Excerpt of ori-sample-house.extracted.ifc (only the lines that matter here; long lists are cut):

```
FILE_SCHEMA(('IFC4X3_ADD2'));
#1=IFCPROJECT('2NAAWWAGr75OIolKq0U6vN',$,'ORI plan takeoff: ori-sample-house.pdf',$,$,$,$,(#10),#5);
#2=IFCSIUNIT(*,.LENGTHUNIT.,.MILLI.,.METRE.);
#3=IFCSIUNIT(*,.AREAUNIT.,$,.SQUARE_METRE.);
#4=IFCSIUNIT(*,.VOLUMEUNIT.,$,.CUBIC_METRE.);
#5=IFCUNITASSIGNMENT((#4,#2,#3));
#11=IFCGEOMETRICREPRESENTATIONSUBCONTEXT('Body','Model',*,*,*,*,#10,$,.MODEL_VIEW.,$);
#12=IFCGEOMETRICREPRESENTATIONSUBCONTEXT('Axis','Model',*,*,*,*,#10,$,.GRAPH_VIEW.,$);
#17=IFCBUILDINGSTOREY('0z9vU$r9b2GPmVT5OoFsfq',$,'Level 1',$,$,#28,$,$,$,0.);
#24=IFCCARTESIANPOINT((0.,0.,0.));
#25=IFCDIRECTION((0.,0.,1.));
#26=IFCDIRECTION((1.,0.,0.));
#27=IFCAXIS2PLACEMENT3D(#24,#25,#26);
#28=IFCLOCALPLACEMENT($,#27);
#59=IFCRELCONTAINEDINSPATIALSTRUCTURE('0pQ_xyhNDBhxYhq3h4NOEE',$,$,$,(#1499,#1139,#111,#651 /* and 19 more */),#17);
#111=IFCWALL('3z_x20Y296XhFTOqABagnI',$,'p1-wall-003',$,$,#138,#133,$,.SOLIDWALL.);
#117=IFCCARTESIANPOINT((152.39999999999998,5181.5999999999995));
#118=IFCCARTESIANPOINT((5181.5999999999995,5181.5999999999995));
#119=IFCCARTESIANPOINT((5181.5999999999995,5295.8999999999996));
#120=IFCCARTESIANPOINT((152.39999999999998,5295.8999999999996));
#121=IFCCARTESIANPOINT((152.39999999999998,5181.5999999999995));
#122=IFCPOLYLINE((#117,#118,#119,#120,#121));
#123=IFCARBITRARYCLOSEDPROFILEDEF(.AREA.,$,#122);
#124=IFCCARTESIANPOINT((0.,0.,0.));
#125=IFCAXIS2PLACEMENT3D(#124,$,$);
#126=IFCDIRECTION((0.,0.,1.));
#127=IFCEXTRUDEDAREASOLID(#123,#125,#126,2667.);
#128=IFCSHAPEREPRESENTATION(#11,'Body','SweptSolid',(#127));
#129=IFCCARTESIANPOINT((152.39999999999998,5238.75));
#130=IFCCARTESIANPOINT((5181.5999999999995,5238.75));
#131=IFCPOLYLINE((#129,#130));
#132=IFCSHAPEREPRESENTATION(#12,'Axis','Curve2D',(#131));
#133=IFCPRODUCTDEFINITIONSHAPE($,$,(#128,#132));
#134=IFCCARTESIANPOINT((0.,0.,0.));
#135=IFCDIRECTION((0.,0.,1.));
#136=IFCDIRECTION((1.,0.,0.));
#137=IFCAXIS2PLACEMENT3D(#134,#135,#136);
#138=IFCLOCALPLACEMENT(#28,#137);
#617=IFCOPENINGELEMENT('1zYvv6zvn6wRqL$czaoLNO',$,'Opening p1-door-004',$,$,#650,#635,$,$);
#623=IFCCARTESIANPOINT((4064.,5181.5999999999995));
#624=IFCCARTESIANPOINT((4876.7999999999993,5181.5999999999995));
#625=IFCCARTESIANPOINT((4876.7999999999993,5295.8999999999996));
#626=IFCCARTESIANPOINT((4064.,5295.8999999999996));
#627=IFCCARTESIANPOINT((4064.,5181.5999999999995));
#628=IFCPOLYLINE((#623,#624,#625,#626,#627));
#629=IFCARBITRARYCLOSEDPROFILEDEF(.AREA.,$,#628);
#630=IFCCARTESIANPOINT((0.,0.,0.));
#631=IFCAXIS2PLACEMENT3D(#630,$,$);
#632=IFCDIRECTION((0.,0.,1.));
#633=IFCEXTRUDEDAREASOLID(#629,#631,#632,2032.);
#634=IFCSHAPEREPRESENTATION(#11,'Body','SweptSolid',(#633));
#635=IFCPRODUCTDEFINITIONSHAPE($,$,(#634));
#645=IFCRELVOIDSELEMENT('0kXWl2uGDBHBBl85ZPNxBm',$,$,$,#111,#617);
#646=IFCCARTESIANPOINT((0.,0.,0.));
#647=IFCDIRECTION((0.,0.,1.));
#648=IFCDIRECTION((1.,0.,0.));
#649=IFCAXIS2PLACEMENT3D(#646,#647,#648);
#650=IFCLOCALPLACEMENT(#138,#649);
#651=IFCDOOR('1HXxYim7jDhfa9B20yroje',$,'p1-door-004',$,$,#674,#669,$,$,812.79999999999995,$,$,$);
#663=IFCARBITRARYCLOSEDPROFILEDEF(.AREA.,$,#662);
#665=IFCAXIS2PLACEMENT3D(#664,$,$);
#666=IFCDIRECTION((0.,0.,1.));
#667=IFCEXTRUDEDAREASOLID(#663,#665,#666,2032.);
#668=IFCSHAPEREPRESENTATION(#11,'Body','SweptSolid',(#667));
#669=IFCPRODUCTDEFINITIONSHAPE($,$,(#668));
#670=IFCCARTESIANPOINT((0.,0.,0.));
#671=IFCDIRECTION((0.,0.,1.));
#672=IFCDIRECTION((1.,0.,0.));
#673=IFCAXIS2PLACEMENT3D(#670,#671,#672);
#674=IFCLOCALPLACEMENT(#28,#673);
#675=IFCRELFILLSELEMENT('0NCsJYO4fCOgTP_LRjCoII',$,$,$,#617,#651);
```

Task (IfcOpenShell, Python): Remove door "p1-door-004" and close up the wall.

```python
import ifcopenshell
import ifcopenshell.api.feature
import ifcopenshell.api.root
import ifcopenshell.geom
import ifcopenshell.util.shape

model = ifcopenshell.open("ori-sample-house.extracted.ifc")
settings = ifcopenshell.geom.settings()


def volume(element):
    """Net volume in cubic metres, openings subtracted."""
    shape = ifcopenshell.geom.create_shape(settings, element)
    return ifcopenshell.util.shape.get_volume(shape.geometry)


door = model.by_id(651)
opening = door.FillsVoids[0].RelatingOpeningElement
wall = opening.VoidsElements[0].RelatingBuildingElement
before = volume(wall)

ifcopenshell.api.root.remove_product(model, product=door)
ifcopenshell.api.feature.remove_feature(model, feature=opening)

after = volume(wall)

print(f"wall volume {before:.3f} -> {after:.3f} m3")

model.write("ori-sample-house.extracted_v2.ifc")
```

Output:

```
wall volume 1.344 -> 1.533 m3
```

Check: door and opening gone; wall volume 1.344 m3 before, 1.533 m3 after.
